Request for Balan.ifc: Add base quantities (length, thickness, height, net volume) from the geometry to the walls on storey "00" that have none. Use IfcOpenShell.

First a look at what the model holds.

```python
import ifcopenshell
import ifcopenshell.util.element
import ifcopenshell.util.unit

model = ifcopenshell.open("Balan.ifc")
print(model.schema)
for unit_type in ("LENGTHUNIT", "AREAUNIT", "VOLUMEUNIT"):
    print(unit_type, ifcopenshell.util.unit.calculate_unit_scale(model, unit_type))
storey = next(s for s in model.by_type("IfcBuildingStorey") if s.Name == "00")
walls = [e for e in ifcopenshell.util.element.get_decomposition(storey) if e.is_a("IfcWall")]
for e in sorted(walls, key=lambda e: e.id()):
    print(e.id(), e.is_a(), e.Name, list(ifcopenshell.util.element.get_psets(e, qtos_only=True)), sep=" | ")
```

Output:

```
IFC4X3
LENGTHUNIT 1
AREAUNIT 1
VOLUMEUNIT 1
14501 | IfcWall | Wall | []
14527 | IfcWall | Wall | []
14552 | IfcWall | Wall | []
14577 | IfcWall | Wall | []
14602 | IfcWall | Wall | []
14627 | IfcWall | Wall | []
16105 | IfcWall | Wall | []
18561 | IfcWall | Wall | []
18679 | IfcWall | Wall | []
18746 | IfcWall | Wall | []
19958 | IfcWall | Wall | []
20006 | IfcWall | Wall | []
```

```python
import ifcopenshell
import ifcopenshell.api.pset
import ifcopenshell.geom
import ifcopenshell.util.element
import ifcopenshell.util.shape
import ifcopenshell.util.unit

model = ifcopenshell.open("Balan.ifc")
unit_scale = ifcopenshell.util.unit.calculate_unit_scale(model)
volume_scale = ifcopenshell.util.unit.calculate_unit_scale(model, "VOLUMEUNIT")
settings = ifcopenshell.geom.settings()

storey = next(s for s in model.by_type("IfcBuildingStorey") if s.Name == "00")
walls = [e for e in ifcopenshell.util.element.get_decomposition(storey) if e.is_a("IfcWall")]

for e in sorted(walls, key=lambda e: e.id()):
    if ifcopenshell.util.element.get_psets(e, qtos_only=True, should_inherit=False):
        continue
    # Geometry comes back in metres, in the element's own axes.
    shape = ifcopenshell.geom.create_shape(settings, e)
    values = {
        "Length": ifcopenshell.util.shape.get_x(shape.geometry) / unit_scale,
        "Width": ifcopenshell.util.shape.get_y(shape.geometry) / unit_scale,
        "Height": ifcopenshell.util.shape.get_z(shape.geometry) / unit_scale,
        "NetVolume": ifcopenshell.util.shape.get_volume(shape.geometry) / volume_scale,
    }
    qto = ifcopenshell.api.pset.add_qto(model, product=e, name="Qto_WallBaseQuantities")
    ifcopenshell.api.pset.edit_qto(model, qto=qto, properties=values)
    print(e.id(), {k: round(v, 3) for k, v in values.items()})

model.write("Balan_rev.ifc")
```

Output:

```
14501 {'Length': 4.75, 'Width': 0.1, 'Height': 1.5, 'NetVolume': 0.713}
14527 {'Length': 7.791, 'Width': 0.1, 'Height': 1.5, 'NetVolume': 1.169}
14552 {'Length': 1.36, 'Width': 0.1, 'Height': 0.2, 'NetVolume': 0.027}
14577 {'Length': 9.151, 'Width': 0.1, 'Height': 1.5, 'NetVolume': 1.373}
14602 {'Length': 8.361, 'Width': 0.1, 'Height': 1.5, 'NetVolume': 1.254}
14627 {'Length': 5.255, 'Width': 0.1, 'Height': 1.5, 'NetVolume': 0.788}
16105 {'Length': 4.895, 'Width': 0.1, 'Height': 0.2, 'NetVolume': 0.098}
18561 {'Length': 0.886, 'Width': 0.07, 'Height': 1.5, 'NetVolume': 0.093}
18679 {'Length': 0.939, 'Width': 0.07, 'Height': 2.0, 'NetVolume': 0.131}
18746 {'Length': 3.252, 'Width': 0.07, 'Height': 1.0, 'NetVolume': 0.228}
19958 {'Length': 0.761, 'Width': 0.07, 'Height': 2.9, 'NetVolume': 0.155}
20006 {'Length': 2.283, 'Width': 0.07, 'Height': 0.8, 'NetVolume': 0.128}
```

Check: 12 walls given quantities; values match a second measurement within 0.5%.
